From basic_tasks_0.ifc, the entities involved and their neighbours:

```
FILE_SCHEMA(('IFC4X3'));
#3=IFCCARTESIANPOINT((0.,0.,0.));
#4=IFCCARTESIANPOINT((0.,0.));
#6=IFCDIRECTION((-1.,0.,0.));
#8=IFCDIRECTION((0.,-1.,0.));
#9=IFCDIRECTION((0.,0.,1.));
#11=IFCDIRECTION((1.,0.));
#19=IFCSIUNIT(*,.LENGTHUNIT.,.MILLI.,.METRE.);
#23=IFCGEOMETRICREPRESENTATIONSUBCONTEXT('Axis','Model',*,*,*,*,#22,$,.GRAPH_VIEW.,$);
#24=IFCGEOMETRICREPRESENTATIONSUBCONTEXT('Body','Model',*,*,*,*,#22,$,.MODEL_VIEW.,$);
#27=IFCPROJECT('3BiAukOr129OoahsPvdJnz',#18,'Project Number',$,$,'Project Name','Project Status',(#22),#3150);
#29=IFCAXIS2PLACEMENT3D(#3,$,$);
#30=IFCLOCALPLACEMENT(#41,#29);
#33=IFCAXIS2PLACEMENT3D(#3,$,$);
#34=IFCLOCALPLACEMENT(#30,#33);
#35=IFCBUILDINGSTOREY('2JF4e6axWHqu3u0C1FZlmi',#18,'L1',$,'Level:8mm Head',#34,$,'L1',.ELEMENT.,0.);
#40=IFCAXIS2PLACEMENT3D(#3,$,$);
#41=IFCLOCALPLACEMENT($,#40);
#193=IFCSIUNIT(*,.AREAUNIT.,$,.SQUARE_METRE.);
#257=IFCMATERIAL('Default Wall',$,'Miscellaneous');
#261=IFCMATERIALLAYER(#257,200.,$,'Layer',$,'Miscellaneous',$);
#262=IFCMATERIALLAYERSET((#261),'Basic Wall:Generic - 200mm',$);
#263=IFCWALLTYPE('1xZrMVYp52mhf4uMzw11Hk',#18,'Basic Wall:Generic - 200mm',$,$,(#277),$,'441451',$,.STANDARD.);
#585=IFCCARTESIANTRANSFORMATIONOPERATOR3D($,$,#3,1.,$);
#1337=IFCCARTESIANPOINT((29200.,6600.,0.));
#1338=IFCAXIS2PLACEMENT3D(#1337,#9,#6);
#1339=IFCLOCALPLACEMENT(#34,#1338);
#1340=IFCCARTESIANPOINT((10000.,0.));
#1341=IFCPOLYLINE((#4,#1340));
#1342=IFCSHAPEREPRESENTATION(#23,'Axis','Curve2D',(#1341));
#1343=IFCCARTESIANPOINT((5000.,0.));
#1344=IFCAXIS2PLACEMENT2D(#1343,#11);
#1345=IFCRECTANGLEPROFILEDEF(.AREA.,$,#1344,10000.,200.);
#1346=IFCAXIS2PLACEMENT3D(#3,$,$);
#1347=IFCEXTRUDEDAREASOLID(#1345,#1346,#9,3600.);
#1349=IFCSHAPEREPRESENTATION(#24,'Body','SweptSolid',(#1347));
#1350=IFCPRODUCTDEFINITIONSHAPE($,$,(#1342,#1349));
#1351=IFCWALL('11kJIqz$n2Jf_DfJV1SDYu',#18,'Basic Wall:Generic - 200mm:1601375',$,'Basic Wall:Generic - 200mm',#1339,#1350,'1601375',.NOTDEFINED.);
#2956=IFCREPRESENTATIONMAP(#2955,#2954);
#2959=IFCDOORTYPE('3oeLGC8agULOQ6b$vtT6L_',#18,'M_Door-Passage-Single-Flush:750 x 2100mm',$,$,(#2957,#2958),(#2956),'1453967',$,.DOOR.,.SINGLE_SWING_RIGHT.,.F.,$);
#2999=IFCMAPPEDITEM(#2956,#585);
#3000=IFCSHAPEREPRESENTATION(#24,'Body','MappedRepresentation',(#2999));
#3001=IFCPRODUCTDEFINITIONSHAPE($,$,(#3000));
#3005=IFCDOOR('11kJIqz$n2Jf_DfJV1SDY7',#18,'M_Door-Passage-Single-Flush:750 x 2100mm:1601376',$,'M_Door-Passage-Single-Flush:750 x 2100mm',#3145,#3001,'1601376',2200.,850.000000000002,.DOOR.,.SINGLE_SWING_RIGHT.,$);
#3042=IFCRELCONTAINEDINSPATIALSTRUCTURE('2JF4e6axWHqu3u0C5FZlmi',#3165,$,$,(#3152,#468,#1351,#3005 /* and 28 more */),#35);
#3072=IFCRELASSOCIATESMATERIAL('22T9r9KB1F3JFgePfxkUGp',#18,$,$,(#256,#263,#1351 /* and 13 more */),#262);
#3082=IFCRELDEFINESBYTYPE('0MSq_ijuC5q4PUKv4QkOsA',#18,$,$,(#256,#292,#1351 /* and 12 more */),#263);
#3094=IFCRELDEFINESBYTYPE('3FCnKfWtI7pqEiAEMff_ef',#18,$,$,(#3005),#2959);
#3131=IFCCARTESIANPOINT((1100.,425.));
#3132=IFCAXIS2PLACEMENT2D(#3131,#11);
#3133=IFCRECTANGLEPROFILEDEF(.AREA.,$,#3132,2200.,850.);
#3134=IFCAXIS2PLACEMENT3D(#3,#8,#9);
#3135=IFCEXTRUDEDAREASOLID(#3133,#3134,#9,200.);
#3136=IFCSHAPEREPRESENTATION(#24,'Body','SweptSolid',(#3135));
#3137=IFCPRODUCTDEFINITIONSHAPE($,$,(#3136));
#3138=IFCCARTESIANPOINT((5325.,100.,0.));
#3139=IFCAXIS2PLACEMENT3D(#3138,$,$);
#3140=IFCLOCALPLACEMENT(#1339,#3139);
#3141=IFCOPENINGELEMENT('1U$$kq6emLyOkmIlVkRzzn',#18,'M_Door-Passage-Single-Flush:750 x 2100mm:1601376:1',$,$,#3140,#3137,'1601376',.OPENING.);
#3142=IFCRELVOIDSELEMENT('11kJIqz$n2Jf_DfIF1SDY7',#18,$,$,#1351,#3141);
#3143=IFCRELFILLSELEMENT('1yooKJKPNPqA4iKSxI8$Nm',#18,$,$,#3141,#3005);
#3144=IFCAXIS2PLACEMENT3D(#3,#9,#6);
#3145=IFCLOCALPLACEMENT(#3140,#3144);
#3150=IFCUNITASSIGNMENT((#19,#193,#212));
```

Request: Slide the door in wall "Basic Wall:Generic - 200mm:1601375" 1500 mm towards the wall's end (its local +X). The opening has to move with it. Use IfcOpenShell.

```python
import ifcopenshell
import ifcopenshell.api.geometry
import ifcopenshell.util.placement

model = ifcopenshell.open("basic_tasks_0.ifc")

door = model.by_guid("11kJIqz$n2Jf_DfJV1SDY7")
opening = door.FillsVoids[0].RelatingOpeningElement
wall = opening.VoidsElements[0].RelatingBuildingElement

wall_matrix = ifcopenshell.util.placement.get_local_placement(wall.ObjectPlacement)
shift = wall_matrix[:3, 0] * 1500.0
before = ifcopenshell.util.placement.get_local_placement(door.ObjectPlacement)[:3, 3].copy()

# The door is placed relative to its opening, so it follows when the opening moves.
matrix = ifcopenshell.util.placement.get_local_placement(opening.ObjectPlacement)
matrix[:3, 3] += shift
ifcopenshell.api.geometry.edit_object_placement(
    model, product=opening, matrix=matrix, is_si=False, should_transform_children=True
)

after = ifcopenshell.util.placement.get_local_placement(door.ObjectPlacement)[:3, 3]
print("door moved by", (after - before).round(3) + 0.0)

model.write("basic_tasks_0_updated.ifc")
```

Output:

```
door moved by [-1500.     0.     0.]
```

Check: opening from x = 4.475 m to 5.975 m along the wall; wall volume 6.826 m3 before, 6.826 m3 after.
